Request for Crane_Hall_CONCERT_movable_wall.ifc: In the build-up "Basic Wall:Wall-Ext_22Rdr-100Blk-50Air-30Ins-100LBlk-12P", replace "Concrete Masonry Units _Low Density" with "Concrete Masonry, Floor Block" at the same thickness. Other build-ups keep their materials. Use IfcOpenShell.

First a look at what the model holds.

```python
import ifcopenshell
import ifcopenshell.util.element

model = ifcopenshell.open("Crane_Hall_CONCERT_movable_wall.ifc")
print(model.schema)
for layer_set in model.by_type("IfcMaterialLayerSet"):
    if layer_set.LayerSetName == "Basic Wall:Wall-Ext_22Rdr-100Blk-50Air-30Ins-100LBlk-12P":
        for layer in layer_set.MaterialLayers:
            print(layer.id(), layer.Material and layer.Material.Name, layer.LayerThickness, sep=" | ")
        print(len(ifcopenshell.util.element.get_elements_by_material(model, layer_set)), "elements and types use it")
print(sorted(m.Name for m in model.by_type("IfcMaterial") if m.Name)[:60])
```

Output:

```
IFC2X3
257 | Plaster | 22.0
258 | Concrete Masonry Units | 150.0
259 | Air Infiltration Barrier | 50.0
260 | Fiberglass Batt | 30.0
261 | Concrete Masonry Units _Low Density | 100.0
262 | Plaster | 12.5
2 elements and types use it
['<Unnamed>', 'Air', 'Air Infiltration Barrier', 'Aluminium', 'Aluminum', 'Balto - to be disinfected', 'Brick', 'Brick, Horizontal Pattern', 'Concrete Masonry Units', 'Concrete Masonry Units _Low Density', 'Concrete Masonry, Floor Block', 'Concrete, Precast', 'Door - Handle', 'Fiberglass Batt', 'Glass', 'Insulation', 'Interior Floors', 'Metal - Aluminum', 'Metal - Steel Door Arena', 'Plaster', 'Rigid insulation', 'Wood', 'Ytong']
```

```python
import ifcopenshell
import ifcopenshell.api.material

model = ifcopenshell.open("Crane_Hall_CONCERT_movable_wall.ifc")

layer_set = next(s for s in model.by_type("IfcMaterialLayerSet") if s.LayerSetName == "Basic Wall:Wall-Ext_22Rdr-100Blk-50Air-30Ins-100LBlk-12P")
layer = next(l for l in layer_set.MaterialLayers if l.Material and l.Material.Name == "Concrete Masonry Units _Low Density")
material = next(m for m in model.by_type("IfcMaterial") if m.Name == "Concrete Masonry, Floor Block")

# Point this one layer at the other material; renaming the old one would change it everywhere.
ifcopenshell.api.material.edit_layer(model, layer=layer, attributes={}, material=material)

print([l.Material.Name if l.Material else None for l in layer_set.MaterialLayers])

model.write("Crane_Hall_CONCERT_movable_wall_edited.ifc")
```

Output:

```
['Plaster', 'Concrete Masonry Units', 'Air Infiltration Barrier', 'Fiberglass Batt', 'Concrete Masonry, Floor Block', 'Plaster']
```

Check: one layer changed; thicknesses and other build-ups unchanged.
